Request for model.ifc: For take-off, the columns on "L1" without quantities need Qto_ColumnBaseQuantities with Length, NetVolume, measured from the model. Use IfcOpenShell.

First a look at what the model holds.

```python
import ifcopenshell
import ifcopenshell.util.element
import ifcopenshell.util.unit

model = ifcopenshell.open("model.ifc")
print(model.schema)
for unit_type in ("LENGTHUNIT", "AREAUNIT", "VOLUMEUNIT"):
    print(unit_type, ifcopenshell.util.unit.calculate_unit_scale(model, unit_type))
storey = next(s for s in model.by_type("IfcBuildingStorey") if s.Name == "L1")
columns = [e for e in ifcopenshell.util.element.get_decomposition(storey) if e.is_a("IfcColumn")]
for e in sorted(columns, key=lambda e: e.id()):
    print(e.id(), e.is_a(), e.Name, list(ifcopenshell.util.element.get_psets(e, qtos_only=True)), sep=" | ")
```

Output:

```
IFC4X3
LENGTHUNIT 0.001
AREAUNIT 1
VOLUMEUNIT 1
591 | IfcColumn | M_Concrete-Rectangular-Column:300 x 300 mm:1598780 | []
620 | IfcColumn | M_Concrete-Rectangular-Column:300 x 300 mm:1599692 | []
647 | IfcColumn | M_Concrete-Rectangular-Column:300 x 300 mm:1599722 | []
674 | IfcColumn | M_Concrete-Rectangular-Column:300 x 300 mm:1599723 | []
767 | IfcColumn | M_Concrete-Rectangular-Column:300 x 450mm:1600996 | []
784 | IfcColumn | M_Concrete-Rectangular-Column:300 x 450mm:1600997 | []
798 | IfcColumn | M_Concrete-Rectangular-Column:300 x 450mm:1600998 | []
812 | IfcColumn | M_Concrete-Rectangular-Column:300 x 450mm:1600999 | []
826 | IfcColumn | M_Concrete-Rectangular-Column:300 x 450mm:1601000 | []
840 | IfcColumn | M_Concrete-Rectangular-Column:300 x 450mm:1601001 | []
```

```python
import ifcopenshell
import ifcopenshell.api.pset
import ifcopenshell.geom
import ifcopenshell.util.element
import ifcopenshell.util.shape
import ifcopenshell.util.unit

model = ifcopenshell.open("model.ifc")
unit_scale = ifcopenshell.util.unit.calculate_unit_scale(model)
volume_scale = ifcopenshell.util.unit.calculate_unit_scale(model, "VOLUMEUNIT")
settings = ifcopenshell.geom.settings()

storey = next(s for s in model.by_type("IfcBuildingStorey") if s.Name == "L1")
columns = [e for e in ifcopenshell.util.element.get_decomposition(storey) if e.is_a("IfcColumn")]

for e in sorted(columns, key=lambda e: e.id()):
    if ifcopenshell.util.element.get_psets(e, qtos_only=True, should_inherit=False):
        continue
    # Geometry comes back in metres, in the element's own axes.
    shape = ifcopenshell.geom.create_shape(settings, e)
    values = {
        "Length": ifcopenshell.util.shape.get_z(shape.geometry) / unit_scale,
        "NetVolume": ifcopenshell.util.shape.get_volume(shape.geometry) / volume_scale,
    }
    qto = ifcopenshell.api.pset.add_qto(model, product=e, name="Qto_ColumnBaseQuantities")
    ifcopenshell.api.pset.edit_qto(model, qto=qto, properties=values)
    print(e.id(), {k: round(v, 3) for k, v in values.items()})

model.write("model_v2.ifc")
```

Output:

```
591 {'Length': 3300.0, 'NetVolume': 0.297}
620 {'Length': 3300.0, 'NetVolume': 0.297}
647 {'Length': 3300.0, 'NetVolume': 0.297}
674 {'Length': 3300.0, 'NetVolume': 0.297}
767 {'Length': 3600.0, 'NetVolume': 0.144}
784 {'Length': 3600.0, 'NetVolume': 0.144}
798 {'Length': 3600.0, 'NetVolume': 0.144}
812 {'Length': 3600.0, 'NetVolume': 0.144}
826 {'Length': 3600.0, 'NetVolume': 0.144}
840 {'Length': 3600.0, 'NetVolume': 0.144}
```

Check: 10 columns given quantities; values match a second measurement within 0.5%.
